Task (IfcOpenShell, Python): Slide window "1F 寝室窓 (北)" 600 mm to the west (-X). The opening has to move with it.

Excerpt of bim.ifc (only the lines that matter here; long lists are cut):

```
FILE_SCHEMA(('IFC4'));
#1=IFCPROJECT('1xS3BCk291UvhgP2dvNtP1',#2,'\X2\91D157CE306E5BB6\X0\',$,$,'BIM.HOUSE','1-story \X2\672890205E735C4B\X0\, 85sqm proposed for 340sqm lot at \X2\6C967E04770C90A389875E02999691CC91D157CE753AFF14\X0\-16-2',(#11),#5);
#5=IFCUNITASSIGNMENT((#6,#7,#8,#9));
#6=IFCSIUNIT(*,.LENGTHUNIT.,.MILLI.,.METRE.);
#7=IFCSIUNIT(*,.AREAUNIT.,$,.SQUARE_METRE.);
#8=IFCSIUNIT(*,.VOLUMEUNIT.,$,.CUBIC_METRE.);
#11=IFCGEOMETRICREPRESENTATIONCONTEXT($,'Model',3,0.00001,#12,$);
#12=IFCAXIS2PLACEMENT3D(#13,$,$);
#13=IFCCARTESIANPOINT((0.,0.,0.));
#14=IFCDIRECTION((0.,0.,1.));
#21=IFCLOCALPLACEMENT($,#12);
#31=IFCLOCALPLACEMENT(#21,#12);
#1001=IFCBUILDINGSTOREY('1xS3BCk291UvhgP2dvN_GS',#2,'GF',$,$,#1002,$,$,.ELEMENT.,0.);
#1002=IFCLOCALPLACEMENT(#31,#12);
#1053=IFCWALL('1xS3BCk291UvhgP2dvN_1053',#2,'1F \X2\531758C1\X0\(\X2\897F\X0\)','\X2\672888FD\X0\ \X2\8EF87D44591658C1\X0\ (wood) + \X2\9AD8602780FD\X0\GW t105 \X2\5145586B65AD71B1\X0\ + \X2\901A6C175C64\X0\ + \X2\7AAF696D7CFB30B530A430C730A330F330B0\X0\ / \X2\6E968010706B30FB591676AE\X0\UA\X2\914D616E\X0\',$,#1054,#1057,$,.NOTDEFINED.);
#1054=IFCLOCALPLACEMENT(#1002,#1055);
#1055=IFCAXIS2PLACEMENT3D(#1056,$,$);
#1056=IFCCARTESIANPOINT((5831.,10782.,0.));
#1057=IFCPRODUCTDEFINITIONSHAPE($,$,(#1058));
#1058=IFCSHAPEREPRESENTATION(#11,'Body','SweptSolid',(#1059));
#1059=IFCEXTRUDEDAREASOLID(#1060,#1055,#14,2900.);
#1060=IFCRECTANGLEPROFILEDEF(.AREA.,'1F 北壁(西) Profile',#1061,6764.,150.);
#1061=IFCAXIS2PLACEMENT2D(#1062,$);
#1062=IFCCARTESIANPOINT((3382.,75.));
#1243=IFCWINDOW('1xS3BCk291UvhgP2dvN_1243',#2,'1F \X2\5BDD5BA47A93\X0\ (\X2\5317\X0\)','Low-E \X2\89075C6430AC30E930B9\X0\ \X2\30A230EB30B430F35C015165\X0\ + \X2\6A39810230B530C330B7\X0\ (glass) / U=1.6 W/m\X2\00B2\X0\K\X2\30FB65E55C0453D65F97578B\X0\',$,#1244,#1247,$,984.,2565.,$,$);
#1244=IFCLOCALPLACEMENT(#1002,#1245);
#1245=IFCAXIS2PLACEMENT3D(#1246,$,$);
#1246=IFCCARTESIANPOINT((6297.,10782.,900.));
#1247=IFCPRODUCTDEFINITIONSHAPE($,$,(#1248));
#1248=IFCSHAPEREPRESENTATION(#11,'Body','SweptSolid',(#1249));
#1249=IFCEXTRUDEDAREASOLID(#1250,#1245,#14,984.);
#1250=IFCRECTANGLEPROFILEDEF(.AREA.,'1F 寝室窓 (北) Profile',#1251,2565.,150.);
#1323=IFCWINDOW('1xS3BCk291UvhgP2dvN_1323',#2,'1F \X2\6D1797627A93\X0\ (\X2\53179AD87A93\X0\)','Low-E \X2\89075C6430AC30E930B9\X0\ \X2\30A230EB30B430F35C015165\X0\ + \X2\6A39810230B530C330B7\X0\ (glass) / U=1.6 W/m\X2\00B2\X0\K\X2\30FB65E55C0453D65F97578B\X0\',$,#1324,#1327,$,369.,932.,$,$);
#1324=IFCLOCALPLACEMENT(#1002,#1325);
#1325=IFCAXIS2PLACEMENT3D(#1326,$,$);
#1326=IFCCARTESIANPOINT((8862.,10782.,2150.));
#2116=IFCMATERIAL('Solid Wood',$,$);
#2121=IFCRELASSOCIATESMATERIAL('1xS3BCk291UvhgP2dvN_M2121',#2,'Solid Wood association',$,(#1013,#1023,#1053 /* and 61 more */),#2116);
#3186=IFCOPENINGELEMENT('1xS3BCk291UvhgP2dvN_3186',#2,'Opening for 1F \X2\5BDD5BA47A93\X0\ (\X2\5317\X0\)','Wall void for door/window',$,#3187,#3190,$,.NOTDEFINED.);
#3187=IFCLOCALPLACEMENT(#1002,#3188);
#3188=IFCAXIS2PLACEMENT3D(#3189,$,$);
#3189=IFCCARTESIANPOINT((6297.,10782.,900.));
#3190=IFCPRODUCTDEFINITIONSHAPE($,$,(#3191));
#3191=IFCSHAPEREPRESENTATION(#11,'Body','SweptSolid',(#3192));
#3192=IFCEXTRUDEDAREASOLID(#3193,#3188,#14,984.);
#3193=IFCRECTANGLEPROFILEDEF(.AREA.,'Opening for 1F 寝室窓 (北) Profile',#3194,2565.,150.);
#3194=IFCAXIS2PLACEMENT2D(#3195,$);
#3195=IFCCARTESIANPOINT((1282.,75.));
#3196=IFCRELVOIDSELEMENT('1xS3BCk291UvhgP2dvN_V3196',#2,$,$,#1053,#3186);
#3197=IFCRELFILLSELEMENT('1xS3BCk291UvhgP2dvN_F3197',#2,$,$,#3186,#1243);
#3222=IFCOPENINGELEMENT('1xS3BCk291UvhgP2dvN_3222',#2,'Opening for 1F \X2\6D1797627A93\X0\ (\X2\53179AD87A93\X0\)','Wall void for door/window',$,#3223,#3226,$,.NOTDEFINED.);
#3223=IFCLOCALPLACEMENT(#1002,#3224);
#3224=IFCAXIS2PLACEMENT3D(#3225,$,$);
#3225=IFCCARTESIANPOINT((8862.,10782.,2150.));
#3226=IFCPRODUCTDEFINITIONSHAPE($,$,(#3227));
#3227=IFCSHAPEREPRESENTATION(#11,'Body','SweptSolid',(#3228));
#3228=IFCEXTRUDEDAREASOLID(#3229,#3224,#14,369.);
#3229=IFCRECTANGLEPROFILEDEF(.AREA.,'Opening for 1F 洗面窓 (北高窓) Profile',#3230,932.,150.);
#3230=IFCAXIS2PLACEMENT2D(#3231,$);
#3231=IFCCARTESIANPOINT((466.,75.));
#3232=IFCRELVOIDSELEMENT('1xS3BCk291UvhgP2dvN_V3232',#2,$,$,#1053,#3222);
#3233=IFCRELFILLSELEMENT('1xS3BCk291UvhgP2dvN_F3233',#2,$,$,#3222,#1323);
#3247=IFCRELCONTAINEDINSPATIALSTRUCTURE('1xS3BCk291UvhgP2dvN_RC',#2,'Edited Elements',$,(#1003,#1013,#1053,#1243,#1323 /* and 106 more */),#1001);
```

```python
import ifcopenshell
import ifcopenshell.api.geometry
import ifcopenshell.util.placement

model = ifcopenshell.open("bim.ifc")

window = model.by_id(1243)
opening = window.FillsVoids[0].RelatingOpeningElement
wall = opening.VoidsElements[0].RelatingBuildingElement

wall_matrix = ifcopenshell.util.placement.get_local_placement(wall.ObjectPlacement)
shift = wall_matrix[:3, 0] * -600.0
before = ifcopenshell.util.placement.get_local_placement(window.ObjectPlacement)[:3, 3].copy()

# The window is not placed relative to its opening, so move both.
for product in (opening, window):
    matrix = ifcopenshell.util.placement.get_local_placement(product.ObjectPlacement)
    matrix[:3, 3] += shift
    ifcopenshell.api.geometry.edit_object_placement(model, product=product, matrix=matrix, is_si=False)

after = ifcopenshell.util.placement.get_local_placement(window.ObjectPlacement)[:3, 3]
print("window moved by", (after - before).round(3) + 0.0)

model.write("bim_rev.ifc")
```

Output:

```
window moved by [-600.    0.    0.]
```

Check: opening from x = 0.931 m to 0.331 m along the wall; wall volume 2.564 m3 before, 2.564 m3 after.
